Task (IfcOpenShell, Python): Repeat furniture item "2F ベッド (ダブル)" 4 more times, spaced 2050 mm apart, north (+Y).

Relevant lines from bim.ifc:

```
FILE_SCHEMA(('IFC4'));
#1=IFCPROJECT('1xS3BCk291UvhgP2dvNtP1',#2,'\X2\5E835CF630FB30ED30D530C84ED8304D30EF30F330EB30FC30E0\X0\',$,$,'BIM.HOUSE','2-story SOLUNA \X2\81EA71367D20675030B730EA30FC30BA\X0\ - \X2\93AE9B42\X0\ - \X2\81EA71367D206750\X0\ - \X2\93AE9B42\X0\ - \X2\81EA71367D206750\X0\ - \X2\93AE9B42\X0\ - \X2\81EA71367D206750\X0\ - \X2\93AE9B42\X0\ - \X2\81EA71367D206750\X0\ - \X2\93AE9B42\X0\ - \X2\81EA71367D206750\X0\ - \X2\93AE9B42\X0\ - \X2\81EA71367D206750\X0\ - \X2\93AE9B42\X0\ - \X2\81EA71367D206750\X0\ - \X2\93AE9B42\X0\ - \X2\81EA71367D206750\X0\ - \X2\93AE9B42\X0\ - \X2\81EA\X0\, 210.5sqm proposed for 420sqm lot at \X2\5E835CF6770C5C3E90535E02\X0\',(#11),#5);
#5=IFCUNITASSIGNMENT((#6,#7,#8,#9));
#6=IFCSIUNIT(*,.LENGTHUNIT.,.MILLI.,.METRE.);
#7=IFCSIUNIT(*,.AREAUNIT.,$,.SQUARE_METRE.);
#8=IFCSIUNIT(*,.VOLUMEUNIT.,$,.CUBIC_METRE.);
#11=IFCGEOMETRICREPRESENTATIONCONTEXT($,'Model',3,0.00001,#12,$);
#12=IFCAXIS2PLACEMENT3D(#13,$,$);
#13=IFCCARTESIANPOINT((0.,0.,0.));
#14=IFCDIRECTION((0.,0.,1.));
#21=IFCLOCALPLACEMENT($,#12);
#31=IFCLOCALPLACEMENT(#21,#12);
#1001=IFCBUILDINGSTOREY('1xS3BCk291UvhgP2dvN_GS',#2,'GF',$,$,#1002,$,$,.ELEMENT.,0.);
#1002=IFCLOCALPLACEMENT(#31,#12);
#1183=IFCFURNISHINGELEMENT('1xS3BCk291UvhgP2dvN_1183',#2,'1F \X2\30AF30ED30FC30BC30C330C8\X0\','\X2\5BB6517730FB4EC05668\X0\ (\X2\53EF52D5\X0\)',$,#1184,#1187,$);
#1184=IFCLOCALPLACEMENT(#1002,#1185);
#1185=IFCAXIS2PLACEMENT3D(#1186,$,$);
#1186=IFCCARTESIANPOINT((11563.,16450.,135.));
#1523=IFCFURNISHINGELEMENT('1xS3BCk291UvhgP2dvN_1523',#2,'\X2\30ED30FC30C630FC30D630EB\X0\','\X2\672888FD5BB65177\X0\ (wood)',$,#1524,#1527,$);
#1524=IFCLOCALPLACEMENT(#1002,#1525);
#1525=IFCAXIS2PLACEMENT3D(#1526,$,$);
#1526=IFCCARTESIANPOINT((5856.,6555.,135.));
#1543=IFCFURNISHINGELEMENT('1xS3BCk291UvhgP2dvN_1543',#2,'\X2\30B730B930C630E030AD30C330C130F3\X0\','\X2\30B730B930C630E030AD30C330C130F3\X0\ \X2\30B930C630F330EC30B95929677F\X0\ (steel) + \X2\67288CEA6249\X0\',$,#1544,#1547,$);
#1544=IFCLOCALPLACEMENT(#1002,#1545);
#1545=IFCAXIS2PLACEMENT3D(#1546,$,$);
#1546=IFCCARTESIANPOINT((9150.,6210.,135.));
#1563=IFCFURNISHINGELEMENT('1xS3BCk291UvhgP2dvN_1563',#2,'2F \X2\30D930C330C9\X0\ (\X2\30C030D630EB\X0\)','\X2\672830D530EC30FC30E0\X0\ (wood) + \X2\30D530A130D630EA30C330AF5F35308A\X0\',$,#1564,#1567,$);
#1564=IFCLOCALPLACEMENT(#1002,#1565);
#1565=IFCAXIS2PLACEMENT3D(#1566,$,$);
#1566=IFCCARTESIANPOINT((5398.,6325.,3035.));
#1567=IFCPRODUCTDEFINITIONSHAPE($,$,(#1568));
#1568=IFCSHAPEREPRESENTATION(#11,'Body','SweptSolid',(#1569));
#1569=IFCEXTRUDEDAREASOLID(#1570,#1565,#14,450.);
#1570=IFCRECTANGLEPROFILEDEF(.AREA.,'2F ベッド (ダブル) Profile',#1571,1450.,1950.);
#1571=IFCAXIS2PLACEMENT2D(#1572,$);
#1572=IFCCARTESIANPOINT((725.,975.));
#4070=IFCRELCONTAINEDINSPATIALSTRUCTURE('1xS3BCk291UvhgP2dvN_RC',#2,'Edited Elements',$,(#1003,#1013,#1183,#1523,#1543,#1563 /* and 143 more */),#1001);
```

```python
import numpy as np
import ifcopenshell
import ifcopenshell.api.geometry
import ifcopenshell.api.root
import ifcopenshell.util.element
import ifcopenshell.util.placement
import ifcopenshell.util.unit

model = ifcopenshell.open("bim.ifc")
unit_scale = ifcopenshell.util.unit.calculate_unit_scale(model)


def reuse_history(source, copy):
    """copy_class also copies each property set's owner history, people and application; keep the originals."""
    for rel in copy.IsDefinedBy:
        if rel.is_a("IfcRelDefinesByProperties") and (history := rel.RelatingPropertyDefinition.OwnerHistory):
            rel.RelatingPropertyDefinition.OwnerHistory = source.OwnerHistory
            ifcopenshell.util.element.remove_deep2(model, history)


source = model.by_id(1563)
base = ifcopenshell.util.placement.get_local_placement(source.ObjectPlacement)
step = np.array([0.0, 1.0, 0.0]) * 2.05 / unit_scale

for i in range(1, 5):
    copy = ifcopenshell.api.root.copy_class(model, product=source)
    copy.Representation = ifcopenshell.util.element.copy_deep(
        model, source.Representation, exclude=["IfcGeometricRepresentationContext", "IfcRepresentationMap"]
    )
    reuse_history(source, copy)
    matrix = base.copy()
    matrix[:3, 3] += i * step
    print("added at", matrix[:3, 3].round(3) + 0.0)
    ifcopenshell.api.geometry.edit_object_placement(model, product=copy, matrix=matrix, is_si=False)

model.write("bim_updated.ifc")
```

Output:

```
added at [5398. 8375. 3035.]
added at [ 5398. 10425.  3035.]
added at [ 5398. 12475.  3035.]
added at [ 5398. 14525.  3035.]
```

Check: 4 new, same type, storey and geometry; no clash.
